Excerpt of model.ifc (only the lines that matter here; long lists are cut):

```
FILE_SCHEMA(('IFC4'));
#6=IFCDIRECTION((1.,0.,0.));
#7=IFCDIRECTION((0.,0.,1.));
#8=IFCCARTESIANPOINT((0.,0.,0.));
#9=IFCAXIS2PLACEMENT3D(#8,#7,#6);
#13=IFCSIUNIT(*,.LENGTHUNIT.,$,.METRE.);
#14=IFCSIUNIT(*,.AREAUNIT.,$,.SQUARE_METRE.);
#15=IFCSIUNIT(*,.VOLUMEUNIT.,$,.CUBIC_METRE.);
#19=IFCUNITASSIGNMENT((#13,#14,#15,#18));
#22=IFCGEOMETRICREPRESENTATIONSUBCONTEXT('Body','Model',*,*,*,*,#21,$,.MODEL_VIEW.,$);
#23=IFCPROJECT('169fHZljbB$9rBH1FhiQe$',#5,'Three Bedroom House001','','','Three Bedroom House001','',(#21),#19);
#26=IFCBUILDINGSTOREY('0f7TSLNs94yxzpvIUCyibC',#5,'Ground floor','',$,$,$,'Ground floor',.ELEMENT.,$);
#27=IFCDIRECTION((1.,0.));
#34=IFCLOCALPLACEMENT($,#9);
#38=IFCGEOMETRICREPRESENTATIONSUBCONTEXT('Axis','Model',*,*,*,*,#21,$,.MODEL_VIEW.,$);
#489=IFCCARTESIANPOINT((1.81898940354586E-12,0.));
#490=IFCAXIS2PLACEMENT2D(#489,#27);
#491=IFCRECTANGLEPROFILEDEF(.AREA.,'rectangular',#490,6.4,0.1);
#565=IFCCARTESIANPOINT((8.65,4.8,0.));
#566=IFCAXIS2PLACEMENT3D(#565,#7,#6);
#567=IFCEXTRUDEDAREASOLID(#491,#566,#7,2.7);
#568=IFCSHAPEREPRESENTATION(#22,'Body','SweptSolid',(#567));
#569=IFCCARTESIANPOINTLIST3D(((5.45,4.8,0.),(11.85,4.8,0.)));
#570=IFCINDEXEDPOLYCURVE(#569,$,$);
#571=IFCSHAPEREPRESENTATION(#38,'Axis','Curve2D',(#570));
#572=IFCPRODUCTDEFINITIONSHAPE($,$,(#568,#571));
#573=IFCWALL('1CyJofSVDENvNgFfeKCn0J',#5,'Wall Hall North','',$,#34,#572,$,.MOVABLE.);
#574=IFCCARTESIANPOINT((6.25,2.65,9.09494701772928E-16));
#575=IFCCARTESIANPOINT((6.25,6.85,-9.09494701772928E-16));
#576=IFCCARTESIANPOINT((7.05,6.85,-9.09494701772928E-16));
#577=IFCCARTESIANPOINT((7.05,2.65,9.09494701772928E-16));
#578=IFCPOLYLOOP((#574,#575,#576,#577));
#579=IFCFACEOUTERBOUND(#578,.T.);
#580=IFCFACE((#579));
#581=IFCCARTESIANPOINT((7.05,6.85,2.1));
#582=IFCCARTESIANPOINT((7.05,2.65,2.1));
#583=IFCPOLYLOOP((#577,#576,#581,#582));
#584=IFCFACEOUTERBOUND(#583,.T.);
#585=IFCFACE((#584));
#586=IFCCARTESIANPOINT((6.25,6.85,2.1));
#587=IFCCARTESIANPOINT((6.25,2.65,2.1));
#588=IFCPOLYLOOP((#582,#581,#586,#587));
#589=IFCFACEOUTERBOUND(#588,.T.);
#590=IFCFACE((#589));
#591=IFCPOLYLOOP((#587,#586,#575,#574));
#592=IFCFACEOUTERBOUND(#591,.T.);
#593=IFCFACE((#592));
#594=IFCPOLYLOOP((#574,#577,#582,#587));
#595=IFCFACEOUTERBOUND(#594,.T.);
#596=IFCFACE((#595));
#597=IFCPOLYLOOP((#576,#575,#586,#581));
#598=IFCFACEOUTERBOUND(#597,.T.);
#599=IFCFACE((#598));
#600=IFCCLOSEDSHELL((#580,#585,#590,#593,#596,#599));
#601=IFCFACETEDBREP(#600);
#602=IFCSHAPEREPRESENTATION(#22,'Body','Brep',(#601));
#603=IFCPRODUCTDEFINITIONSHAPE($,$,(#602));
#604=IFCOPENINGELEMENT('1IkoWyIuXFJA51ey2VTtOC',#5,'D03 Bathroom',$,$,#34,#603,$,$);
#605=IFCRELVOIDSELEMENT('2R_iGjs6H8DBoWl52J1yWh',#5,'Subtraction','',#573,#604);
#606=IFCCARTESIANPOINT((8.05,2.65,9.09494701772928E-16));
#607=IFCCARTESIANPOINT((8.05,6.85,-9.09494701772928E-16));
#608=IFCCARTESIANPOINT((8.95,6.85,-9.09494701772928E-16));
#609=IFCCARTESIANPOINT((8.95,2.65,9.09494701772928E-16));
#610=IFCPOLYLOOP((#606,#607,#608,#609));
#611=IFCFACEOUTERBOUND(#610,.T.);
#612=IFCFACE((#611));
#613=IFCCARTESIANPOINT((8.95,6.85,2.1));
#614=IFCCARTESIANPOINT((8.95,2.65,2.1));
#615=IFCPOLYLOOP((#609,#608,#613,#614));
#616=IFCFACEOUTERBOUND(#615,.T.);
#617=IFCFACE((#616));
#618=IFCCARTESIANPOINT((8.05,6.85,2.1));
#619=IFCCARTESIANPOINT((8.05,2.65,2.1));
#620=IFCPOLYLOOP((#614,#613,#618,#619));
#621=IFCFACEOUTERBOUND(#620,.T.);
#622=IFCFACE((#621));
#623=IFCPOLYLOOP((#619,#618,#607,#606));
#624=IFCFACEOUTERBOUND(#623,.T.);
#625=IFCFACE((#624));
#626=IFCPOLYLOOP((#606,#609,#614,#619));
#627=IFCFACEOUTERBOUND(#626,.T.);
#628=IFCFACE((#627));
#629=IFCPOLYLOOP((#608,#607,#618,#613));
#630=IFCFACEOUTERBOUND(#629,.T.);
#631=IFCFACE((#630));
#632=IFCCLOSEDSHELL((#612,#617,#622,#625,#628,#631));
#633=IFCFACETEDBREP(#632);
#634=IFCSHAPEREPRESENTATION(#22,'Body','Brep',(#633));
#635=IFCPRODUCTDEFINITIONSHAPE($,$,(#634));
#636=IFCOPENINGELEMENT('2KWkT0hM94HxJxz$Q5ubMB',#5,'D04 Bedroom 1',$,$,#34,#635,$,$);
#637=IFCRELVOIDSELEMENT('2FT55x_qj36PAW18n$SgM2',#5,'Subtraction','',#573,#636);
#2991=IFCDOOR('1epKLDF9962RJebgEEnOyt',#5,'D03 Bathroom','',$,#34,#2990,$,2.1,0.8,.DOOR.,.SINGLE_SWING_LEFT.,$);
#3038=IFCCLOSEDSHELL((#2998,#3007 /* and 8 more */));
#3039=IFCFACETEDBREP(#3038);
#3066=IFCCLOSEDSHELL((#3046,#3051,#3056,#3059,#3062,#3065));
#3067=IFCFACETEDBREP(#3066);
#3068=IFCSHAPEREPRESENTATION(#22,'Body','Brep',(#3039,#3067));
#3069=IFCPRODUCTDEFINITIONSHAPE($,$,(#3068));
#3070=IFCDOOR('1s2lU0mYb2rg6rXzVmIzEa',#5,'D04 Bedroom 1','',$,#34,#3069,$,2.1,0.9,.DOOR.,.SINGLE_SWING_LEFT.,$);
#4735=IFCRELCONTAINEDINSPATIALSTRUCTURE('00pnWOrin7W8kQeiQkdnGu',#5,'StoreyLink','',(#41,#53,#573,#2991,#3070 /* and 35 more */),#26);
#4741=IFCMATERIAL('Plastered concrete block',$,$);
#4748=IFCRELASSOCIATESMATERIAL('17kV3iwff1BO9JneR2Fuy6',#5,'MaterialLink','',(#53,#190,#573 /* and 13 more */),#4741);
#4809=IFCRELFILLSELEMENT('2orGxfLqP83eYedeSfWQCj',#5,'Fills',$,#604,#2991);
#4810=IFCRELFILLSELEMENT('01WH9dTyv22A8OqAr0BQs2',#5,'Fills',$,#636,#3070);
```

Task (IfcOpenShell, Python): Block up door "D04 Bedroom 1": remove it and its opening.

```python
import ifcopenshell
import ifcopenshell.api.feature
import ifcopenshell.api.root
import ifcopenshell.geom
import ifcopenshell.util.shape

model = ifcopenshell.open("model.ifc")
settings = ifcopenshell.geom.settings()


def volume(element):
    """Net volume in cubic metres, openings subtracted."""
    shape = ifcopenshell.geom.create_shape(settings, element)
    return ifcopenshell.util.shape.get_volume(shape.geometry)


door = model.by_guid("1s2lU0mYb2rg6rXzVmIzEa")
opening = door.FillsVoids[0].RelatingOpeningElement
wall = opening.VoidsElements[0].RelatingBuildingElement
before = volume(wall)

ifcopenshell.api.root.remove_product(model, product=door)
ifcopenshell.api.feature.remove_feature(model, feature=opening)

after = volume(wall)

print(f"wall volume {before:.3f} -> {after:.3f} m3")

model.write("model_rev.ifc")
```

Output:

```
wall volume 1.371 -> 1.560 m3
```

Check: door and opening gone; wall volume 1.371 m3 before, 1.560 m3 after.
